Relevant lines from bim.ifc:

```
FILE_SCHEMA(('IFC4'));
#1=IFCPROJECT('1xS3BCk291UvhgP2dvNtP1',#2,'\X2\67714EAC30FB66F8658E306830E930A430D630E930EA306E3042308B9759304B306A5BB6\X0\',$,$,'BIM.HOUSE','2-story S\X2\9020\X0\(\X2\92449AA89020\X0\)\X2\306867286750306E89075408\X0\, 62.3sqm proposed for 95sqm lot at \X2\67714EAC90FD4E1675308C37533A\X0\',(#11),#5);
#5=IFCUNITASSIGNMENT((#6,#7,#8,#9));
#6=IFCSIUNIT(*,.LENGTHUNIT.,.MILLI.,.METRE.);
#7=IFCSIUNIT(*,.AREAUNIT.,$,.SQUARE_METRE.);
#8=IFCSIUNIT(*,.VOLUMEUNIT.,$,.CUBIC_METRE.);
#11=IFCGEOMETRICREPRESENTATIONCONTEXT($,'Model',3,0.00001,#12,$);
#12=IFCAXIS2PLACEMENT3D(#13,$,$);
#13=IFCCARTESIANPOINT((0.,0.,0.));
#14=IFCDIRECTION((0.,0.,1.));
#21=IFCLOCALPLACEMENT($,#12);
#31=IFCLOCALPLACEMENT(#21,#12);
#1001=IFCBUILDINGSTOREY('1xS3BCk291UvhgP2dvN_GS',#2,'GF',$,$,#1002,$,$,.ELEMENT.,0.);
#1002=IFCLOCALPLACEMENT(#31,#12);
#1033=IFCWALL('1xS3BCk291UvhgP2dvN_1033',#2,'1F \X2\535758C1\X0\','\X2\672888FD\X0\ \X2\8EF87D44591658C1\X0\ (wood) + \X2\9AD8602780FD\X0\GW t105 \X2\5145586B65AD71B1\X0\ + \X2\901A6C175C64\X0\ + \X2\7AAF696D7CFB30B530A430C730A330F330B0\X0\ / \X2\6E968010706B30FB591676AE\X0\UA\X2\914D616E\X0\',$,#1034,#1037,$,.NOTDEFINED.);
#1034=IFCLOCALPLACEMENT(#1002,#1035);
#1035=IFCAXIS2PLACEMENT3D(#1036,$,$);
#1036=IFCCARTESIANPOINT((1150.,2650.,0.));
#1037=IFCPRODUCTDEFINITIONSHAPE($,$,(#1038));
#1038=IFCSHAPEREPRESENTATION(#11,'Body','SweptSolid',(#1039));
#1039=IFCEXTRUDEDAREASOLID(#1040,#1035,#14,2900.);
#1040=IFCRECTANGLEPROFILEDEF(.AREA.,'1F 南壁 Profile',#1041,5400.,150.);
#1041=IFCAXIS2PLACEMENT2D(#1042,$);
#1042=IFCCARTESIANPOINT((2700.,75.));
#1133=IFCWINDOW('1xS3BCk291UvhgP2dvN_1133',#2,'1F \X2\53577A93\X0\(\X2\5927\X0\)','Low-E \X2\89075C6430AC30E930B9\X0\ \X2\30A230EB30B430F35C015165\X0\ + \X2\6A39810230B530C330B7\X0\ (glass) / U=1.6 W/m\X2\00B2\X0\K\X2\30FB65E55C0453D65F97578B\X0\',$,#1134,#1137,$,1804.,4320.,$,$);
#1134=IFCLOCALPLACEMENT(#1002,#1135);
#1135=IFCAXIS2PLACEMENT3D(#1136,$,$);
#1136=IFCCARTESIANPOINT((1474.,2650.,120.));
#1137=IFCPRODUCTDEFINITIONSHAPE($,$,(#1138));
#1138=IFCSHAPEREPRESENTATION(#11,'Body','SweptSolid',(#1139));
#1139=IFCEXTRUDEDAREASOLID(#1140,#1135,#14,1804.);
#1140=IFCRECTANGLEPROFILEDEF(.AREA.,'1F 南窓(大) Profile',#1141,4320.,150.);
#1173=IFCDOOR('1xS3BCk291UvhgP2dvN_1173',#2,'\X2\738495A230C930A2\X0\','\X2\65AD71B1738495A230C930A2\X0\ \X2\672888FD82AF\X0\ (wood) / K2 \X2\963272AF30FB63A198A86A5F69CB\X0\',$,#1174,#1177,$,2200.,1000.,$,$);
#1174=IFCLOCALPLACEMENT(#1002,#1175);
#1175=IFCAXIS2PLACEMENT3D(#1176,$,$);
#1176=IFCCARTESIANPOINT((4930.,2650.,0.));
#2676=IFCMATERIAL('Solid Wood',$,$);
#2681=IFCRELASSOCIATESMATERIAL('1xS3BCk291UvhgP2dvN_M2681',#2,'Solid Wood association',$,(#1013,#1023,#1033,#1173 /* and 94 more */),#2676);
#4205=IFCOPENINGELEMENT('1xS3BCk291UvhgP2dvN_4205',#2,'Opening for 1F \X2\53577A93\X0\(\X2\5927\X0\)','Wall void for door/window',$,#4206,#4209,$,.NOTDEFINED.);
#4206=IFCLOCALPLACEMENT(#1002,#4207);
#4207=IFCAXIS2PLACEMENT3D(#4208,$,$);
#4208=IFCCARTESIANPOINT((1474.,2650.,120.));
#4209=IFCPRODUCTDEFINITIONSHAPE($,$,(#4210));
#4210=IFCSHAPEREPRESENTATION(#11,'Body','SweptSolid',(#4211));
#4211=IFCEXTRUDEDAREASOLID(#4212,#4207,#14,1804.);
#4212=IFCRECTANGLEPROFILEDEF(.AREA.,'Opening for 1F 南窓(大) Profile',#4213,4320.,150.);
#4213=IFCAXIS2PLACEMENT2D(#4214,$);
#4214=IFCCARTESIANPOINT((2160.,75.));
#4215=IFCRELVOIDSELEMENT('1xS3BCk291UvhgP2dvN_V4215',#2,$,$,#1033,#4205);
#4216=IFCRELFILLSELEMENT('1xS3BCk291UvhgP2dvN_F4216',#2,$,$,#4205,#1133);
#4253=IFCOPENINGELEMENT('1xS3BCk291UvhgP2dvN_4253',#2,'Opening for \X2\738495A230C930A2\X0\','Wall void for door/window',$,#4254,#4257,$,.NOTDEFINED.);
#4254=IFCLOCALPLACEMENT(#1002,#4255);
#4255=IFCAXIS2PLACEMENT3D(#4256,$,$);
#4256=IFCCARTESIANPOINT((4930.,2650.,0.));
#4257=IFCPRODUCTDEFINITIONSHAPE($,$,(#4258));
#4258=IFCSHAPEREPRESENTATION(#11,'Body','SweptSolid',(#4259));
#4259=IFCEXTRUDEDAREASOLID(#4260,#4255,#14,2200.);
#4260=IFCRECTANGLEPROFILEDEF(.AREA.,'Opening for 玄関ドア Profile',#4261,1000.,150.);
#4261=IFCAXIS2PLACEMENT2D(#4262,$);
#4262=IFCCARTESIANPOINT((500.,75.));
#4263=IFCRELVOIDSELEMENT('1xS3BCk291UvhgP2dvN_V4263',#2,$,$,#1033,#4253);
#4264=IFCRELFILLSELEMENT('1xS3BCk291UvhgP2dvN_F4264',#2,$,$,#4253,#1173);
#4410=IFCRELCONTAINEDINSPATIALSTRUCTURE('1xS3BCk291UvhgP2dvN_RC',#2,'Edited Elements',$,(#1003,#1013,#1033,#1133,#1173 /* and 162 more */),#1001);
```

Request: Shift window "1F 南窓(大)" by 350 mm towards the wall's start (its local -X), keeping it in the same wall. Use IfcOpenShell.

```python
import ifcopenshell
import ifcopenshell.api.geometry
import ifcopenshell.util.placement
import ifcopenshell.util.unit

model = ifcopenshell.open("bim.ifc")
unit_scale = ifcopenshell.util.unit.calculate_unit_scale(model)

window = model.by_id(1133)
opening = window.FillsVoids[0].RelatingOpeningElement
wall = opening.VoidsElements[0].RelatingBuildingElement

wall_matrix = ifcopenshell.util.placement.get_local_placement(wall.ObjectPlacement)
shift = wall_matrix[:3, 0] * -0.35 / unit_scale
before = ifcopenshell.util.placement.get_local_placement(window.ObjectPlacement)[:3, 3].copy()

# The window is not placed relative to its opening, so move both.
for product in (opening, window):
    matrix = ifcopenshell.util.placement.get_local_placement(product.ObjectPlacement)
    matrix[:3, 3] += shift
    ifcopenshell.api.geometry.edit_object_placement(model, product=product, matrix=matrix, is_si=False)

after = ifcopenshell.util.placement.get_local_placement(window.ObjectPlacement)[:3, 3]
print("window moved by", (after - before).round(3) + 0.0)

model.write("bim_rev.ifc")
```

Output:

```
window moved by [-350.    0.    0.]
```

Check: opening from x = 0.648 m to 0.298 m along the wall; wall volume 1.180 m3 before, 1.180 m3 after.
